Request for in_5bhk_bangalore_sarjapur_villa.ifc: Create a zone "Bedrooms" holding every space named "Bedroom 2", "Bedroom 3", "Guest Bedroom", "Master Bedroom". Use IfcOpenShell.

First a look at what the model holds.

```python
import ifcopenshell

model = ifcopenshell.open("in_5bhk_bangalore_sarjapur_villa.ifc")
print(model.schema)
seen = {}
for space in model.by_type("IfcSpace"):
    seen[space.LongName] = seen.get(space.LongName, 0) + 1
for name, count in sorted(seen.items(), key=str):
    print(count, "x", name)
print("zones:", [z.Name for z in model.by_type("IfcZone")][:20])
```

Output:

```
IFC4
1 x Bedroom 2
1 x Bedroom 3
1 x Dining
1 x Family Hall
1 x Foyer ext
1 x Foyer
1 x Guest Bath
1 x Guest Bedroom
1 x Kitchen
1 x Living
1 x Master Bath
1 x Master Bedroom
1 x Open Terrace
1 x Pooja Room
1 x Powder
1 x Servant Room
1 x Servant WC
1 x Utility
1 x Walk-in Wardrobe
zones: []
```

```python
import ifcopenshell
import ifcopenshell.api.group
import ifcopenshell.api.root

model = ifcopenshell.open("in_5bhk_bangalore_sarjapur_villa.ifc")

names = {"Bedroom 2", "Bedroom 3", "Guest Bedroom", "Master Bedroom"}
spaces = [s for s in model.by_type("IfcSpace") if s.LongName in names]

zone = ifcopenshell.api.root.create_entity(model, ifc_class="IfcZone", name="Bedrooms")
ifcopenshell.api.group.assign_group(model, products=spaces, group=zone)
print(len(spaces), "spaces in", zone.Name)

model.write("in_5bhk_bangalore_sarjapur_villa_rev.ifc")
```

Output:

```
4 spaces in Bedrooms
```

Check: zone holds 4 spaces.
